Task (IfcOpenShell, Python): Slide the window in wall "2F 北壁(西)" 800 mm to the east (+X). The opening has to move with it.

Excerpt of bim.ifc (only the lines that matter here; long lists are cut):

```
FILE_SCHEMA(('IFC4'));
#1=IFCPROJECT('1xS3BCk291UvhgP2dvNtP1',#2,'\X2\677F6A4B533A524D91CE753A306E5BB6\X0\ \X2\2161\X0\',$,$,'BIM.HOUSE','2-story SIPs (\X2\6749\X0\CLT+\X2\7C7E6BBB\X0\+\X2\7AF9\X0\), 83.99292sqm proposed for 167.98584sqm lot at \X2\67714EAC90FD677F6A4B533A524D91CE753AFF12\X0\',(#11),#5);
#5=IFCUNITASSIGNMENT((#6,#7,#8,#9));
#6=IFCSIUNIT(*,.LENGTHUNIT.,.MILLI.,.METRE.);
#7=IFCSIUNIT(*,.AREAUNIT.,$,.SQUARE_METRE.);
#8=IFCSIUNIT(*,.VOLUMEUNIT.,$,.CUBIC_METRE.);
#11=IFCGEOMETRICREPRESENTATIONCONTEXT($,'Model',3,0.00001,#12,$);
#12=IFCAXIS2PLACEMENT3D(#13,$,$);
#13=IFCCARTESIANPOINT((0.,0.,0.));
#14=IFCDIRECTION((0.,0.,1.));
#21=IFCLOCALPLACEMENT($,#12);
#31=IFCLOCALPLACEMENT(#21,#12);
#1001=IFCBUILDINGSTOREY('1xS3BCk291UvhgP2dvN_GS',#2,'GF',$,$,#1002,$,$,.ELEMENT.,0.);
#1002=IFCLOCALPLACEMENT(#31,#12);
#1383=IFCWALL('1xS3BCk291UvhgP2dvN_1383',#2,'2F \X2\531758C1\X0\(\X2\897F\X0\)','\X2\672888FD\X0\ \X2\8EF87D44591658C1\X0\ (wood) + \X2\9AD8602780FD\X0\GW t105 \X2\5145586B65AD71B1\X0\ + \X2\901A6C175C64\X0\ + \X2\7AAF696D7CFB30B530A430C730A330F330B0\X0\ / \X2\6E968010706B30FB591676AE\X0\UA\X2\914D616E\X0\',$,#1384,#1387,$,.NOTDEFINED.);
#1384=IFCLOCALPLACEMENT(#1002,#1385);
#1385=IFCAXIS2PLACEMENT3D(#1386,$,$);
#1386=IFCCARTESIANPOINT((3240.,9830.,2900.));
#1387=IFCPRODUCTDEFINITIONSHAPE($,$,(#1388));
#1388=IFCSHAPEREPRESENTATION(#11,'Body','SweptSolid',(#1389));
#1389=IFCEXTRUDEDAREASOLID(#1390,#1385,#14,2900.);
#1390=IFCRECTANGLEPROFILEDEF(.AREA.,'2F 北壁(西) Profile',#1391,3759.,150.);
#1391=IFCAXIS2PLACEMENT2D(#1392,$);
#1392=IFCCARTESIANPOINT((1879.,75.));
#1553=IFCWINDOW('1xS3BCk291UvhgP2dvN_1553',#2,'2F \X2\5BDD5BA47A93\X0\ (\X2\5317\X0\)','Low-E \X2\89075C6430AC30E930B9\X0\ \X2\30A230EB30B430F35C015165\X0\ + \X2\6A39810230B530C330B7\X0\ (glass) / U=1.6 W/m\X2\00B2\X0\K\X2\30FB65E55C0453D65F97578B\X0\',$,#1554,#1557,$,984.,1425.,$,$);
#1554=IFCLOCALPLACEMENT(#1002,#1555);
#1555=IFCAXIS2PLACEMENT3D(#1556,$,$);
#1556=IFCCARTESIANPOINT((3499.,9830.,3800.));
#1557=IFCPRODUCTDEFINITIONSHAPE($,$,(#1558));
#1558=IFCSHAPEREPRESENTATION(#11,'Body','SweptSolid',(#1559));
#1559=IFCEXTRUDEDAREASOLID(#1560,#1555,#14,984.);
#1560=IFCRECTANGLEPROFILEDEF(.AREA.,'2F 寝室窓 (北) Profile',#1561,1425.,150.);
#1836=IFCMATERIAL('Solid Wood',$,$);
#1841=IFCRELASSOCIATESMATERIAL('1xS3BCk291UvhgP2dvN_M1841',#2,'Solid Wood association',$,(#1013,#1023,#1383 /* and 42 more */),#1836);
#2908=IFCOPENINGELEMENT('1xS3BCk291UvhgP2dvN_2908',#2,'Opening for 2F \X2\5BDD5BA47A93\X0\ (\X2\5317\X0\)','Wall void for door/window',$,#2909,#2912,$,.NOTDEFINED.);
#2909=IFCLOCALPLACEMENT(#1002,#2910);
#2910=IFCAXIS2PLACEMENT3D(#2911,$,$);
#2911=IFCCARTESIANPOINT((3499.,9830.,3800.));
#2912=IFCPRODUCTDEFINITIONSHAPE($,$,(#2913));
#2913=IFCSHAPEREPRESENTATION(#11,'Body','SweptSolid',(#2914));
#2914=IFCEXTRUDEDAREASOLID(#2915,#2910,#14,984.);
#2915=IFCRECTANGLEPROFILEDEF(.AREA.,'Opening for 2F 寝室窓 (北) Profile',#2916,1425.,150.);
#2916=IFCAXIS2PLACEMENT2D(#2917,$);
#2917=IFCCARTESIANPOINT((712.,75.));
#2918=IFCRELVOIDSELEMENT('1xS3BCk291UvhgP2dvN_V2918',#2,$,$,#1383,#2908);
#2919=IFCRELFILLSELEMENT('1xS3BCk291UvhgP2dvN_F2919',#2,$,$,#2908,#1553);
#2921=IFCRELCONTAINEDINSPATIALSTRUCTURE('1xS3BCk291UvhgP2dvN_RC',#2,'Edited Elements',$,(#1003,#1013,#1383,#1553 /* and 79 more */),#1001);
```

```python
import ifcopenshell
import ifcopenshell.api.geometry
import ifcopenshell.util.placement
import ifcopenshell.util.unit

model = ifcopenshell.open("bim.ifc")
unit_scale = ifcopenshell.util.unit.calculate_unit_scale(model)

window = model.by_guid("1xS3BCk291UvhgP2dvN_1553")
opening = window.FillsVoids[0].RelatingOpeningElement
wall = opening.VoidsElements[0].RelatingBuildingElement

wall_matrix = ifcopenshell.util.placement.get_local_placement(wall.ObjectPlacement)
shift = wall_matrix[:3, 0] * 0.8 / unit_scale
before = ifcopenshell.util.placement.get_local_placement(window.ObjectPlacement)[:3, 3].copy()

# The window is not placed relative to its opening, so move both.
for product in (opening, window):
    matrix = ifcopenshell.util.placement.get_local_placement(product.ObjectPlacement)
    matrix[:3, 3] += shift
    ifcopenshell.api.geometry.edit_object_placement(model, product=product, matrix=matrix, is_si=False)

after = ifcopenshell.util.placement.get_local_placement(window.ObjectPlacement)[:3, 3]
print("window moved by", (after - before).round(3) + 0.0)

model.write("bim_rev.ifc")
```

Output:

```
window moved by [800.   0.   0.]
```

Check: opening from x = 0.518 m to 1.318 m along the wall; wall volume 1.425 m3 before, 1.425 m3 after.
